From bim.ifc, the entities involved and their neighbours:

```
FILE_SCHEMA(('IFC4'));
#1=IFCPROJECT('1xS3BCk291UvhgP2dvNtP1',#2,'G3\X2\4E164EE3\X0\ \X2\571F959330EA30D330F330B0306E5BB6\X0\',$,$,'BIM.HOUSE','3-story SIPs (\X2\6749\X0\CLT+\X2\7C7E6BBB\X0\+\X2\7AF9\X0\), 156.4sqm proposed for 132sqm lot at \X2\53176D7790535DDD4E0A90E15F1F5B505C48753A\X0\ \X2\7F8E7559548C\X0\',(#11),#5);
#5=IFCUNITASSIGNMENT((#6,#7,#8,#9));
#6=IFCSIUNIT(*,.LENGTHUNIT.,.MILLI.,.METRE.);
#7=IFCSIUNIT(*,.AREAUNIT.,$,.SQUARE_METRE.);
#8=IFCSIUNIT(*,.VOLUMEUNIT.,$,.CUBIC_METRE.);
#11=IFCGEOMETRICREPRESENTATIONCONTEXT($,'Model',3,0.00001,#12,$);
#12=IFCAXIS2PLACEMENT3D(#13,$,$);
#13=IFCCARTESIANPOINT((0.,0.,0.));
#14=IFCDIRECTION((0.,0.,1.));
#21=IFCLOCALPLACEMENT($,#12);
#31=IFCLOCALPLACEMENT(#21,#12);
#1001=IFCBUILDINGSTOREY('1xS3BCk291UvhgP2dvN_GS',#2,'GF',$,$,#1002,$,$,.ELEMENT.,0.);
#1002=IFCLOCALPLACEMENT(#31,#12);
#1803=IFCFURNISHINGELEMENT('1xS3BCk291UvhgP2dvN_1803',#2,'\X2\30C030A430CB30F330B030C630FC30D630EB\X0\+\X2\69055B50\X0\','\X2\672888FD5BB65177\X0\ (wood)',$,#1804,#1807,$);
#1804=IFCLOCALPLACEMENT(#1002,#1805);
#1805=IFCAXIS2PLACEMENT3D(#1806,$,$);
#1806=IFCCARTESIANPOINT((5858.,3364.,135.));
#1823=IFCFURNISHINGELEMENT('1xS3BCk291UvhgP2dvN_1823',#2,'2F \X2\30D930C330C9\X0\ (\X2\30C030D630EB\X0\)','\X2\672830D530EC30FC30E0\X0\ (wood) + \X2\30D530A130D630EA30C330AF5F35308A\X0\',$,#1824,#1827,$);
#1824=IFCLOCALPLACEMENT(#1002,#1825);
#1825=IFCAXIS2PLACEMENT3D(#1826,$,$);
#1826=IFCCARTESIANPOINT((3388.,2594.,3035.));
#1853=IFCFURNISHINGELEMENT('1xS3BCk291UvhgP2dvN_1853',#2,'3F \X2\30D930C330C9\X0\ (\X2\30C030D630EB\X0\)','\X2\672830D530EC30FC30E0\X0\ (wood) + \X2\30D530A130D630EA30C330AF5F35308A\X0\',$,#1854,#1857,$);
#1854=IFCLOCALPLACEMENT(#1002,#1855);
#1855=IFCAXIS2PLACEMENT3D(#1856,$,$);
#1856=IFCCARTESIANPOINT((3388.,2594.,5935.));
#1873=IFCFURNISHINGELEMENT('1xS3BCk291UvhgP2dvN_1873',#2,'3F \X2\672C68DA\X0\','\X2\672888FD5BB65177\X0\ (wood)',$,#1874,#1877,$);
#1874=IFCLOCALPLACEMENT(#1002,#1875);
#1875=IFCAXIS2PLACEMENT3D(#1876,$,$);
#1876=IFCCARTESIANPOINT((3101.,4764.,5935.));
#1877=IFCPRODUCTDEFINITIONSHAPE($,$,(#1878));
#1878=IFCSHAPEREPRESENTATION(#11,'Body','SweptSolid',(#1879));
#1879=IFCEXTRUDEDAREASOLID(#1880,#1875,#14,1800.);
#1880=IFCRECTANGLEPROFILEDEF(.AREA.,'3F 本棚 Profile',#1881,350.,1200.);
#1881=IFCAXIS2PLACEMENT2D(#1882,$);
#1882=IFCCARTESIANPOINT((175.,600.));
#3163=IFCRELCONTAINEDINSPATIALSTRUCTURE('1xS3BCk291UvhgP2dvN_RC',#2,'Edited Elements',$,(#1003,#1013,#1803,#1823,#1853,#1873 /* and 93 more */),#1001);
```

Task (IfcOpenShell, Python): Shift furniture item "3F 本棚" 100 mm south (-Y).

```python
import ifcopenshell
import ifcopenshell.api.geometry
import ifcopenshell.util.placement

model = ifcopenshell.open("bim.ifc")

item = model.by_id(1873)
matrix = ifcopenshell.util.placement.get_local_placement(item.ObjectPlacement)
matrix[1, 3] -= 100.0
ifcopenshell.api.geometry.edit_object_placement(model, product=item, matrix=matrix, is_si=False)

print(ifcopenshell.util.placement.get_local_placement(item.ObjectPlacement).round(3) + 0.0)

model.write("bim-out.ifc")
```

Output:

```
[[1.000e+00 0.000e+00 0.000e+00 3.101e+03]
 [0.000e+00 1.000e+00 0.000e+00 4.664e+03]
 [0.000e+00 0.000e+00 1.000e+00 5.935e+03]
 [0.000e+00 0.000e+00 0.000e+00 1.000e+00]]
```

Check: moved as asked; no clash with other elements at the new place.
